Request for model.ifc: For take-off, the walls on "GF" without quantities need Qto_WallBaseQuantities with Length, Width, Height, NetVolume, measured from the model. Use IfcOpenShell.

First a look at what the model holds.

```python
import ifcopenshell
import ifcopenshell.util.element
import ifcopenshell.util.unit

model = ifcopenshell.open("model.ifc")
print(model.schema)
for unit_type in ("LENGTHUNIT", "AREAUNIT", "VOLUMEUNIT"):
    print(unit_type, ifcopenshell.util.unit.calculate_unit_scale(model, unit_type))
storey = next(s for s in model.by_type("IfcBuildingStorey") if s.Name == "GF")
walls = [e for e in ifcopenshell.util.element.get_decomposition(storey) if e.is_a("IfcWall")]
for e in sorted(walls, key=lambda e: e.id()):
    print(e.id(), e.is_a(), e.Name, list(ifcopenshell.util.element.get_psets(e, qtos_only=True)), sep=" | ")
```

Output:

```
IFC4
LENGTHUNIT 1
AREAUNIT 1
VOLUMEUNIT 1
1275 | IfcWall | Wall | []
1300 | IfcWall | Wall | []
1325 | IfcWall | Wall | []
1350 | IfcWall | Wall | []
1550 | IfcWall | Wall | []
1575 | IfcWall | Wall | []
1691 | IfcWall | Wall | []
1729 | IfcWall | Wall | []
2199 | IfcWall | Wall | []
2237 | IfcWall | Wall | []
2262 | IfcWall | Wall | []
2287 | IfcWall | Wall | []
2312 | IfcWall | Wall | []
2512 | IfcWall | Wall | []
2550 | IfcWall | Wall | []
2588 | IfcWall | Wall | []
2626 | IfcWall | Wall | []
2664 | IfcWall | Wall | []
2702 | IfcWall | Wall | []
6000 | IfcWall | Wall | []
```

```python
import ifcopenshell
import ifcopenshell.api.pset
import ifcopenshell.geom
import ifcopenshell.util.element
import ifcopenshell.util.shape
import ifcopenshell.util.unit

model = ifcopenshell.open("model.ifc")
unit_scale = ifcopenshell.util.unit.calculate_unit_scale(model)
volume_scale = ifcopenshell.util.unit.calculate_unit_scale(model, "VOLUMEUNIT")
settings = ifcopenshell.geom.settings()

storey = next(s for s in model.by_type("IfcBuildingStorey") if s.Name == "GF")
walls = [e for e in ifcopenshell.util.element.get_decomposition(storey) if e.is_a("IfcWall")]

for e in sorted(walls, key=lambda e: e.id()):
    if ifcopenshell.util.element.get_psets(e, qtos_only=True, should_inherit=False):
        continue
    # Geometry comes back in metres, in the element's own axes.
    shape = ifcopenshell.geom.create_shape(settings, e)
    values = {
        "Length": ifcopenshell.util.shape.get_x(shape.geometry) / unit_scale,
        "Width": ifcopenshell.util.shape.get_y(shape.geometry) / unit_scale,
        "Height": ifcopenshell.util.shape.get_z(shape.geometry) / unit_scale,
        "NetVolume": ifcopenshell.util.shape.get_volume(shape.geometry) / volume_scale,
    }
    qto = ifcopenshell.api.pset.add_qto(model, product=e, name="Qto_WallBaseQuantities")
    ifcopenshell.api.pset.edit_qto(model, qto=qto, properties=values)
    print(e.id(), {k: round(v, 3) for k, v in values.items()})

model.write("model-out.ifc")
```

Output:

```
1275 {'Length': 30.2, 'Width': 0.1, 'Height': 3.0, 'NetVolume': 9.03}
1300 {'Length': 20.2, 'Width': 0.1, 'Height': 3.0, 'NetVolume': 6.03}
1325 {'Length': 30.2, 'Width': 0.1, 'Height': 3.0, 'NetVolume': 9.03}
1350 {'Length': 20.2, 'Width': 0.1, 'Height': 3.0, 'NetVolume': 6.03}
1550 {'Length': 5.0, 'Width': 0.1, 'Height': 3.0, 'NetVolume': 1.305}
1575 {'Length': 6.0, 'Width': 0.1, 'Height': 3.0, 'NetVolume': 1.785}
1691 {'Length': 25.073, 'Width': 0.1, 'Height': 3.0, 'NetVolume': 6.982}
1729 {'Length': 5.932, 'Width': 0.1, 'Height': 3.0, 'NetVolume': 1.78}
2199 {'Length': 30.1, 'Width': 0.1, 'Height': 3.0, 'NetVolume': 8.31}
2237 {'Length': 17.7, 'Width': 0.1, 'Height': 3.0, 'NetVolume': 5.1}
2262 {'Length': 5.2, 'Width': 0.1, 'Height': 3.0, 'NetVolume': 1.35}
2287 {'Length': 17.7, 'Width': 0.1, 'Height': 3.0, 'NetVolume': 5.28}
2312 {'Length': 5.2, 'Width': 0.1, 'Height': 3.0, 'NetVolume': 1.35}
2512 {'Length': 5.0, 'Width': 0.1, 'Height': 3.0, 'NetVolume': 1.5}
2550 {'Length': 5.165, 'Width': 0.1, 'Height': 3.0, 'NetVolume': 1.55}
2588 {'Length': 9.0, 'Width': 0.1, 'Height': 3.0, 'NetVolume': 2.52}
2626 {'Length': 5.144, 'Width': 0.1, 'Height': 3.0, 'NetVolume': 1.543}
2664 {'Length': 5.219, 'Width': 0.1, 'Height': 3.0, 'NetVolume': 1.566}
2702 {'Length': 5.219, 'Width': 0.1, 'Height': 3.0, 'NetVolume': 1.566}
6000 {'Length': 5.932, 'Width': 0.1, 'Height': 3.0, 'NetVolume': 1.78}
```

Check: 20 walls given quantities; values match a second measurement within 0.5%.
